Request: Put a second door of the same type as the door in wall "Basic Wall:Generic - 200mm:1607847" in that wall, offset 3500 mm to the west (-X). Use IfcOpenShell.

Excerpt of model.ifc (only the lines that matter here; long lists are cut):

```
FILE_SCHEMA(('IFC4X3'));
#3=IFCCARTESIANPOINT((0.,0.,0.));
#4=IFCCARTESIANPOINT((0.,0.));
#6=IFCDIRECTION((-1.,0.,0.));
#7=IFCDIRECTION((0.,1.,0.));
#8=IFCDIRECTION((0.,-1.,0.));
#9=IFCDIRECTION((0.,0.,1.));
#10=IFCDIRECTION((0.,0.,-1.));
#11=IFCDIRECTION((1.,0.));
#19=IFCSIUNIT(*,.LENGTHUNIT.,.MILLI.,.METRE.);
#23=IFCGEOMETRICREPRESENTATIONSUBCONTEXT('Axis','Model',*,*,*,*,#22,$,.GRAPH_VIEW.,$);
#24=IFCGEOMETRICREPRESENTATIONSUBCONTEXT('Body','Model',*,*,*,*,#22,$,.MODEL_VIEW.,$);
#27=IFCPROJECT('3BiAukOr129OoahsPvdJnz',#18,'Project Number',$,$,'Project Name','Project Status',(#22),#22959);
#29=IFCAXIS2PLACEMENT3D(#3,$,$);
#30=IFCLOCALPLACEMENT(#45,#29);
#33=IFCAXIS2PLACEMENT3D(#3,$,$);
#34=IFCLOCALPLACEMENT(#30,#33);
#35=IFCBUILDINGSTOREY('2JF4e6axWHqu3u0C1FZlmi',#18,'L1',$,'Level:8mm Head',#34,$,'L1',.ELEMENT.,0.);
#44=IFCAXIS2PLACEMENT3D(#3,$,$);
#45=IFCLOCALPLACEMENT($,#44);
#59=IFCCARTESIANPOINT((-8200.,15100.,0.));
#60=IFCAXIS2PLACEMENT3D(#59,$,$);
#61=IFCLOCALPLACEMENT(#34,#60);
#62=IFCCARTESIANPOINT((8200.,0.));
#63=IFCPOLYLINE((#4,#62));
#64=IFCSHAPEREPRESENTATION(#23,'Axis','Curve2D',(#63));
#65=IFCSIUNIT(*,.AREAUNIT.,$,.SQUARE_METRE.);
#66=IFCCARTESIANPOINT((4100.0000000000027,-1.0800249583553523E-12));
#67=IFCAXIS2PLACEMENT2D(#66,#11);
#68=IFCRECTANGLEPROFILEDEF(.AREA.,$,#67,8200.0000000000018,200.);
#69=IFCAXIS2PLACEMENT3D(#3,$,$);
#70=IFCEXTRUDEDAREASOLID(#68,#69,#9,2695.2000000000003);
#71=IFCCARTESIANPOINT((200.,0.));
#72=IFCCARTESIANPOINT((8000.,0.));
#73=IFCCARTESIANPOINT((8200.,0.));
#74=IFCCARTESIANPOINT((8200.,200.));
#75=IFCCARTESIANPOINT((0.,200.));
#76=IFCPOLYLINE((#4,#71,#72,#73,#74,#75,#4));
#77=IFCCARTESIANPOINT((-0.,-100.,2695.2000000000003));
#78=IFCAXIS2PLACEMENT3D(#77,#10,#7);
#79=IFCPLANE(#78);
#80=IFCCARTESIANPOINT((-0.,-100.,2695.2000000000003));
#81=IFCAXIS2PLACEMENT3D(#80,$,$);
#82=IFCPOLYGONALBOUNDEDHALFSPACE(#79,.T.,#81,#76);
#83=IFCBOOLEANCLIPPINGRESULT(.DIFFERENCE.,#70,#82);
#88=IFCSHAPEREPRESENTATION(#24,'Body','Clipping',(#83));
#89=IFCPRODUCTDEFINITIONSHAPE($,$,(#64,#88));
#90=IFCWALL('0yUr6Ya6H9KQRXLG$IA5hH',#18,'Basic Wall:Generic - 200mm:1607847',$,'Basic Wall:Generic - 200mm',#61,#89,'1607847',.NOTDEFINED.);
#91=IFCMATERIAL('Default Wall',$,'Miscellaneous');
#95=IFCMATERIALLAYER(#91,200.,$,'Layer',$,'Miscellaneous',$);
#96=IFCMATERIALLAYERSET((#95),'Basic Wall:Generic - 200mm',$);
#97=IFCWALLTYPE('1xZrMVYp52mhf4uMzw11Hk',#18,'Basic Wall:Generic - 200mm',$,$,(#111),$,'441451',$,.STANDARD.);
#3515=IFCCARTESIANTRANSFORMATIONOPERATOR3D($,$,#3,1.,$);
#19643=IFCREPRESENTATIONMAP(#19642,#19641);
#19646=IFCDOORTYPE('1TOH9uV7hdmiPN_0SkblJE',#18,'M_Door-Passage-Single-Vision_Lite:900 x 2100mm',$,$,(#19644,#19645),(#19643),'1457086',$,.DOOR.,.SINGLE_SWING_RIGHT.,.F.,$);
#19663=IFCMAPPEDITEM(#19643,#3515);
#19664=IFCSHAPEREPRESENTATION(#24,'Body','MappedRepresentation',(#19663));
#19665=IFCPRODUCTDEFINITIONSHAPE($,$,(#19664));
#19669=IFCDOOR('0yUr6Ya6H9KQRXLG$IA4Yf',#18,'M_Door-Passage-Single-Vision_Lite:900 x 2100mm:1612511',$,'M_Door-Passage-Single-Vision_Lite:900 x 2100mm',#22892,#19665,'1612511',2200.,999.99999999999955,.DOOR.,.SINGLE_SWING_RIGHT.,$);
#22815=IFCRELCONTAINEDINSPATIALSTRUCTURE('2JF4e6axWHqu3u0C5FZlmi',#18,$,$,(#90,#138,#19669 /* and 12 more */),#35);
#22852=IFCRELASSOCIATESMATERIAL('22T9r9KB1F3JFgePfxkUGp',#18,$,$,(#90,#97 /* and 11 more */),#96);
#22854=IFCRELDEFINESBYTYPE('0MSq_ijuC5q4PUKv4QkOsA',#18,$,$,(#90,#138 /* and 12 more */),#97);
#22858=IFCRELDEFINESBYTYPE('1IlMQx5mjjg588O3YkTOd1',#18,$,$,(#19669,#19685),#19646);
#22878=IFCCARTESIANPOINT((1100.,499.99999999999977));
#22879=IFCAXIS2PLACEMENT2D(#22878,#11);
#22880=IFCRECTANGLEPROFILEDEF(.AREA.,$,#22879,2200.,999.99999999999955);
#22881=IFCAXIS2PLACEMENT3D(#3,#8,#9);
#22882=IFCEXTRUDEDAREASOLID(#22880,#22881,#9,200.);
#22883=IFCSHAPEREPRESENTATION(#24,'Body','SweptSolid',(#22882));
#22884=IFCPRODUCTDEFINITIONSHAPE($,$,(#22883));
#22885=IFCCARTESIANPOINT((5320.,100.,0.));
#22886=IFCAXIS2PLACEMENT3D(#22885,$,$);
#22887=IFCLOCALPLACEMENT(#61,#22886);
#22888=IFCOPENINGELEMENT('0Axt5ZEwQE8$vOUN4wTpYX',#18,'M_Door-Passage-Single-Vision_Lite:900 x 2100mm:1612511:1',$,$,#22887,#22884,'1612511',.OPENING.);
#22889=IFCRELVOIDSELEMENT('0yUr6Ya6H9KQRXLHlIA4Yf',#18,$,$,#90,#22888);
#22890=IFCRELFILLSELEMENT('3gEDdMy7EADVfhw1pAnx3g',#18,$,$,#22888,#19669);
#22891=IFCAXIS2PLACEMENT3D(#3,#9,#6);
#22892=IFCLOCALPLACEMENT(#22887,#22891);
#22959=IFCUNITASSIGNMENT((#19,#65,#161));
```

```python
import ifcopenshell
import ifcopenshell.api.feature
import ifcopenshell.api.geometry
import ifcopenshell.api.root
import ifcopenshell.geom
import ifcopenshell.util.element
import ifcopenshell.util.placement
import ifcopenshell.util.shape

model = ifcopenshell.open("model.ifc")
settings = ifcopenshell.geom.settings()


def volume(element):
    """Net volume in cubic metres, openings subtracted."""
    shape = ifcopenshell.geom.create_shape(settings, element)
    return ifcopenshell.util.shape.get_volume(shape.geometry)


def reuse_history(source, copy):
    """copy_class also copies each property set's owner history, people and application; keep the originals."""
    for rel in copy.IsDefinedBy:
        if rel.is_a("IfcRelDefinesByProperties") and (history := rel.RelatingPropertyDefinition.OwnerHistory):
            rel.RelatingPropertyDefinition.OwnerHistory = source.OwnerHistory
            ifcopenshell.util.element.remove_deep2(model, history)


door = model.by_guid("0yUr6Ya6H9KQRXLG$IA4Yf")
opening = door.FillsVoids[0].RelatingOpeningElement
wall = opening.VoidsElements[0].RelatingBuildingElement
before = volume(wall)
shift = ifcopenshell.util.placement.get_local_placement(wall.ObjectPlacement)[:3, 0] * -3500.0

# copy_class copies the void relationship, type, container and properties, but no geometry.
new_opening = ifcopenshell.api.root.copy_class(model, product=opening)
new_opening.Representation = ifcopenshell.util.element.copy_deep(
    model, opening.Representation, exclude=["IfcGeometricRepresentationContext", "IfcRepresentationMap"]
)
new_opening.Name = "M_Door-Passage-Single-Vision_Lite:900 x 2100mm"
new_opening.Tag = None
new_door = ifcopenshell.api.root.copy_class(model, product=door)
new_door.Representation = ifcopenshell.util.element.copy_deep(
    model, door.Representation, exclude=["IfcGeometricRepresentationContext", "IfcRepresentationMap"]
)
new_door.Name = "M_Door-Passage-Single-Vision_Lite:900 x 2100mm"
new_door.Tag = None
reuse_history(door, new_door)
ifcopenshell.api.feature.add_filling(model, opening=new_opening, element=new_door)

for old, new in ((opening, new_opening), (door, new_door)):
    matrix = ifcopenshell.util.placement.get_local_placement(old.ObjectPlacement)
    matrix[:3, 3] += shift
    ifcopenshell.api.geometry.edit_object_placement(model, product=new, matrix=matrix, is_si=False)

after = volume(wall)

print(f"wall volume {before:.3f} -> {after:.3f} m3")

model.write("model-out.ifc")
```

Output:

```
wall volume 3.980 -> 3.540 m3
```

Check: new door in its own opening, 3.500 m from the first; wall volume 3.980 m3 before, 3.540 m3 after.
